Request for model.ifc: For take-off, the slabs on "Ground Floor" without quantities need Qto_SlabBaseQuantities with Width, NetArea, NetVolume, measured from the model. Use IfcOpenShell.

First a look at what the model holds.

```python
import ifcopenshell
import ifcopenshell.util.element
import ifcopenshell.util.unit

model = ifcopenshell.open("model.ifc")
print(model.schema)
for unit_type in ("LENGTHUNIT", "AREAUNIT", "VOLUMEUNIT"):
    print(unit_type, ifcopenshell.util.unit.calculate_unit_scale(model, unit_type))
storey = next(s for s in model.by_type("IfcBuildingStorey") if s.Name == "Ground Floor")
slabs = [e for e in ifcopenshell.util.element.get_decomposition(storey) if e.is_a("IfcSlab")]
for e in sorted(slabs, key=lambda e: e.id()):
    print(e.id(), e.is_a(), e.Name, list(ifcopenshell.util.element.get_psets(e, qtos_only=True)), sep=" | ")
```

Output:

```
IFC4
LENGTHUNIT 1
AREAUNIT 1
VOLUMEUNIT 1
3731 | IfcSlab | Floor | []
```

```python
import ifcopenshell
import ifcopenshell.api.pset
import ifcopenshell.geom
import ifcopenshell.util.element
import ifcopenshell.util.shape
import ifcopenshell.util.unit

model = ifcopenshell.open("model.ifc")
unit_scale = ifcopenshell.util.unit.calculate_unit_scale(model)
area_scale = ifcopenshell.util.unit.calculate_unit_scale(model, "AREAUNIT")
volume_scale = ifcopenshell.util.unit.calculate_unit_scale(model, "VOLUMEUNIT")
settings = ifcopenshell.geom.settings()

storey = next(s for s in model.by_type("IfcBuildingStorey") if s.Name == "Ground Floor")
slabs = [e for e in ifcopenshell.util.element.get_decomposition(storey) if e.is_a("IfcSlab")]

for e in sorted(slabs, key=lambda e: e.id()):
    if ifcopenshell.util.element.get_psets(e, qtos_only=True, should_inherit=False):
        continue
    # Geometry comes back in metres, in the element's own axes.
    shape = ifcopenshell.geom.create_shape(settings, e)
    values = {
        "Width": ifcopenshell.util.shape.get_z(shape.geometry) / unit_scale,
        "NetArea": ifcopenshell.util.shape.get_footprint_area(shape.geometry) / area_scale,
        "NetVolume": ifcopenshell.util.shape.get_volume(shape.geometry) / volume_scale,
    }
    qto = ifcopenshell.api.pset.add_qto(model, product=e, name="Qto_SlabBaseQuantities")
    ifcopenshell.api.pset.edit_qto(model, qto=qto, properties=values)
    print(e.id(), {k: round(v, 3) for k, v in values.items()})

model.write("model-out.ifc")
```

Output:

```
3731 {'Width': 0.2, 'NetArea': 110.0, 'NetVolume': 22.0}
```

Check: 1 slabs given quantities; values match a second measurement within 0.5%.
